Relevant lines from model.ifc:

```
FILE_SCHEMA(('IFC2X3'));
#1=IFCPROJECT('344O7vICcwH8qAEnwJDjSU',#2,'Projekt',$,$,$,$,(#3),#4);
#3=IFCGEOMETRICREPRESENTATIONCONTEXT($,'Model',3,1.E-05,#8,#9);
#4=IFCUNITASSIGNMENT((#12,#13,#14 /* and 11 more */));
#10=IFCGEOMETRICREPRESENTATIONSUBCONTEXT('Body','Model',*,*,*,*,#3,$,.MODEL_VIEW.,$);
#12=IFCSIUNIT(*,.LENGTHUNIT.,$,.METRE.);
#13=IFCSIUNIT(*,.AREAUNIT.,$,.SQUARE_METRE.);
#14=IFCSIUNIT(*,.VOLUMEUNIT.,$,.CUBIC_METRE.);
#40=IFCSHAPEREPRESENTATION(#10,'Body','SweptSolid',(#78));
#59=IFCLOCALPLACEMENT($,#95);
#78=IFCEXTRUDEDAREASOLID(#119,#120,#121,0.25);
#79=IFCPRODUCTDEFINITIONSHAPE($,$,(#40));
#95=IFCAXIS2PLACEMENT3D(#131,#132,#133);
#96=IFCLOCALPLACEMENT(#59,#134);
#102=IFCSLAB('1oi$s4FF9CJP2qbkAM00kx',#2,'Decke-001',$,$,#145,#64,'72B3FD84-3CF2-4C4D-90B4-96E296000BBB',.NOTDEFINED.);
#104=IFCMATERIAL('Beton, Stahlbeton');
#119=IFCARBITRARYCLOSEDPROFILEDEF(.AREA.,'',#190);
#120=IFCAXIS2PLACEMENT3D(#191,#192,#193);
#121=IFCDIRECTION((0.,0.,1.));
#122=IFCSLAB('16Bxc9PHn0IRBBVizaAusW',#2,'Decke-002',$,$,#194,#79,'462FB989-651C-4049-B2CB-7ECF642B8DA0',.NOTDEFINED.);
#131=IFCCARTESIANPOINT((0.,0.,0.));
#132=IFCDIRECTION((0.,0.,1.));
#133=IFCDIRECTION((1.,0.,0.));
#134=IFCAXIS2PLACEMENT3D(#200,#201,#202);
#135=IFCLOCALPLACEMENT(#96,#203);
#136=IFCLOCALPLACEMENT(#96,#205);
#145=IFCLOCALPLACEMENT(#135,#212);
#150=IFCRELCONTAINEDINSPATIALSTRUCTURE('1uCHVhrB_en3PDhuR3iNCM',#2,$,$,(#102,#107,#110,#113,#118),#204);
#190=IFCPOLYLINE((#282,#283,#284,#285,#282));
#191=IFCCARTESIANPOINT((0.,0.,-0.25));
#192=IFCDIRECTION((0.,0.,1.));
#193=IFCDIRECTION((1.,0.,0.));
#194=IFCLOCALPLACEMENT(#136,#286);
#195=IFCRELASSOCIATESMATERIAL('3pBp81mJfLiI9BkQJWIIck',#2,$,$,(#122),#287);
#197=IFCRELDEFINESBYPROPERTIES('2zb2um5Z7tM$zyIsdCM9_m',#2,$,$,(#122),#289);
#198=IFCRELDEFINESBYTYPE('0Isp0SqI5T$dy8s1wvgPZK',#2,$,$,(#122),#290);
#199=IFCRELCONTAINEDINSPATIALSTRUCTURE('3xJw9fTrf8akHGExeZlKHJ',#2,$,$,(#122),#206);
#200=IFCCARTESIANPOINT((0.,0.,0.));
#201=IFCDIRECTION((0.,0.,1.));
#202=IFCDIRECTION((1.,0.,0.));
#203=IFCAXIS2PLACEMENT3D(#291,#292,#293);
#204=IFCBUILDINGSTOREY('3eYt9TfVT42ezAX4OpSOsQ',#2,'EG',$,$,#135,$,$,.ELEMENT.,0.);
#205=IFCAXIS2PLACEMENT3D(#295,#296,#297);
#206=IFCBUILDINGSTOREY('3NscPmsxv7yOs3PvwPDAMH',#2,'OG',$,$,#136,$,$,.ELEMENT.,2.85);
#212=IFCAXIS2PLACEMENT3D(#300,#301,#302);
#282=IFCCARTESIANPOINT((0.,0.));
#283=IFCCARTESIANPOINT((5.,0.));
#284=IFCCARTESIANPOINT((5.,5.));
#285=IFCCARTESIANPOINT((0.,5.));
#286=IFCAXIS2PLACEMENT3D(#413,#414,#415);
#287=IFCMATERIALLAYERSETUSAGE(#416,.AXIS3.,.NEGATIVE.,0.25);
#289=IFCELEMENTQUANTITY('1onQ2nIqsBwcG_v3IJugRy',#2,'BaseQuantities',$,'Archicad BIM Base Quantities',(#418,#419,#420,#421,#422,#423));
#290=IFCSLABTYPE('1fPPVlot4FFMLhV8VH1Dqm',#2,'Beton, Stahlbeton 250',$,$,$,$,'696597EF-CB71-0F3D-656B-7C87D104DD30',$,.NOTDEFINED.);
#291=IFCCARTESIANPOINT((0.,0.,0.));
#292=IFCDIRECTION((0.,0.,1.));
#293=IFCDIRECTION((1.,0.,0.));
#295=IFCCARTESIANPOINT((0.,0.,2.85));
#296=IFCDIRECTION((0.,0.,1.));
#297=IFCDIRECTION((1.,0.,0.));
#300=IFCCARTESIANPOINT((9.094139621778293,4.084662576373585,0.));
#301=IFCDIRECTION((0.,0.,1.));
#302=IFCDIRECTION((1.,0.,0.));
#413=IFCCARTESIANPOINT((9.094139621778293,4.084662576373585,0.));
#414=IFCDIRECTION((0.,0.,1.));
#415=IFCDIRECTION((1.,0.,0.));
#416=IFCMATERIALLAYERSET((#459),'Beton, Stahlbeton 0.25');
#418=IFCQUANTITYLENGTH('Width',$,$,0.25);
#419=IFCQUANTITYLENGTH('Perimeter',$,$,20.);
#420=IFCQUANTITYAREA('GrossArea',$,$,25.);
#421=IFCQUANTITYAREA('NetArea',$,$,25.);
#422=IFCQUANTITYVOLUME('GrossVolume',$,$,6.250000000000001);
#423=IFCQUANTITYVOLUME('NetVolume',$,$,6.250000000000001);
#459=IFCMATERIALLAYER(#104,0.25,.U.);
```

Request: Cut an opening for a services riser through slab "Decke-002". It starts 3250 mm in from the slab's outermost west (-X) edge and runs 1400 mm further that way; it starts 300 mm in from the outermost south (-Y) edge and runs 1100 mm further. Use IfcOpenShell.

```python
import numpy as np
import ifcopenshell
import ifcopenshell.api.feature
import ifcopenshell.api.geometry
import ifcopenshell.api.pset
import ifcopenshell.api.root
import ifcopenshell.geom
import ifcopenshell.util.element
import ifcopenshell.util.placement
import ifcopenshell.util.representation
import ifcopenshell.util.shape
import ifcopenshell.util.unit

model = ifcopenshell.open("model.ifc")
unit_scale = ifcopenshell.util.unit.calculate_unit_scale(model)
area_scale = ifcopenshell.util.unit.calculate_unit_scale(model, "AREAUNIT")
volume_scale = ifcopenshell.util.unit.calculate_unit_scale(model, "VOLUMEUNIT")
settings = ifcopenshell.geom.settings()


def volume(element):
    """Net volume in cubic metres, openings subtracted."""
    shape = ifcopenshell.geom.create_shape(settings, element)
    return ifcopenshell.util.shape.get_volume(shape.geometry)


slab = model.by_guid("16Bxc9PHn0IRBBVizaAusW")
before = volume(slab)

# Extent in the slab's own axes, in metres. The edges named are its -X and -Y sides.
slab_shape = ifcopenshell.geom.create_shape(settings, slab)
vertices = ifcopenshell.util.shape.get_vertices(slab_shape.geometry)
x_min, y_min, bottom = vertices.min(axis=0)
top = vertices[:, 2].max()

opening = ifcopenshell.api.root.create_entity(model, ifc_class="IfcOpeningElement", name="Services riser opening")
context = ifcopenshell.util.representation.get_context(model, "Model", "Body", "MODEL_VIEW")
width, depth = 1.4, 1.1
outline = [(0.0, 0.0), (width, 0.0), (width, depth), (0.0, depth), (0.0, 0.0)]
# Overshoot both faces by 50 mm so the cut is clean.
shape = ifcopenshell.api.geometry.add_slab_representation(
    model, context=context, depth=top - bottom + 0.1, polyline=outline
)
ifcopenshell.api.geometry.assign_representation(model, product=opening, representation=shape)

matrix = ifcopenshell.util.placement.get_local_placement(slab.ObjectPlacement)
matrix[:, 3] = matrix @ np.append(np.array([x_min + 3.25, y_min + 0.3, bottom - 0.05]) / unit_scale, 1.0)
ifcopenshell.api.geometry.edit_object_placement(model, product=opening, matrix=matrix, is_si=False)
ifcopenshell.api.feature.add_feature(model, feature=opening, element=slab)

after = volume(slab)

# Update the slab's stored quantities.
qto = model.by_id(ifcopenshell.util.element.get_pset(slab, "BaseQuantities", should_inherit=False)["id"])
ifcopenshell.api.pset.edit_qto(model, qto=qto, properties={
    "NetArea": after / (top - bottom) / area_scale,
    "NetVolume": after / volume_scale,
})

print(f"slab volume {before:.3f} -> {after:.3f} m3")

model.write("model_updated.ifc")
```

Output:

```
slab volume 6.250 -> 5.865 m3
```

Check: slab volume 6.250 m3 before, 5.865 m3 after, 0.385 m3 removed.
